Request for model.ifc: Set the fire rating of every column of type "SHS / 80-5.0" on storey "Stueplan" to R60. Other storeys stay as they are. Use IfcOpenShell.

First a look at what the model holds.

```python
import ifcopenshell
import ifcopenshell.util.element

model = ifcopenshell.open("model.ifc")
print(model.schema)
storey = next(s for s in model.by_type("IfcBuildingStorey") if s.Name == "Stueplan")
columns = [e for e in ifcopenshell.util.element.get_decomposition(storey) if e.is_a("IfcColumn")]
seen = {}
for e in columns:
    element_type = ifcopenshell.util.element.get_type(e)
    key = (element_type.Name if element_type != e and element_type else None, ifcopenshell.util.element.get_pset(e, "Pset_ColumnCommon", "FireRating"))
    seen[key] = seen.get(key, 0) + 1
for (name, value), count in sorted(seen.items(), key=str):
    print(count, "x", name, "|", value)
```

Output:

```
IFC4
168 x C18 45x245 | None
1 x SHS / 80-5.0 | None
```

```python
import ifcopenshell
import ifcopenshell.api.pset
import ifcopenshell.util.element

model = ifcopenshell.open("model.ifc")

storey = next(s for s in model.by_type("IfcBuildingStorey") if s.Name == "Stueplan")
columns = [e for e in ifcopenshell.util.element.get_decomposition(storey) if e.is_a("IfcColumn")]

count = 0
for e in columns:
    element_type = ifcopenshell.util.element.get_type(e)
    if element_type in (None, e) or element_type.Name != "SHS / 80-5.0":
        continue
    # add_pset returns the element's existing set when there is one.
    pset = ifcopenshell.api.pset.add_pset(model, product=e, name="Pset_ColumnCommon")
    ifcopenshell.api.pset.edit_pset(model, pset=pset, properties={"FireRating": "R60"})
    count += 1

print(count, "columns updated")

model.write("model_updated.ifc")
```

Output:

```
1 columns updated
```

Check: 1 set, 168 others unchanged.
